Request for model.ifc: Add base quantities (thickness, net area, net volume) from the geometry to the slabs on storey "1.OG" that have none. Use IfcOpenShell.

First a look at what the model holds.

```python
import ifcopenshell
import ifcopenshell.util.element
import ifcopenshell.util.unit

model = ifcopenshell.open("model.ifc")
print(model.schema)
for unit_type in ("LENGTHUNIT", "AREAUNIT", "VOLUMEUNIT"):
    print(unit_type, ifcopenshell.util.unit.calculate_unit_scale(model, unit_type))
storey = next(s for s in model.by_type("IfcBuildingStorey") if s.Name == "1.OG")
slabs = [e for e in ifcopenshell.util.element.get_decomposition(storey) if e.is_a("IfcSlab")]
for e in sorted(slabs, key=lambda e: e.id()):
    print(e.id(), e.is_a(), e.Name, list(ifcopenshell.util.element.get_psets(e, qtos_only=True)), sep=" | ")
```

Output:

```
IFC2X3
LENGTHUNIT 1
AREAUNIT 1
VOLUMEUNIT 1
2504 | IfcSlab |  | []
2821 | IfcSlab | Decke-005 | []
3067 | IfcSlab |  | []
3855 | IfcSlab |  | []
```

```python
import ifcopenshell
import ifcopenshell.api.pset
import ifcopenshell.geom
import ifcopenshell.util.element
import ifcopenshell.util.shape
import ifcopenshell.util.unit

model = ifcopenshell.open("model.ifc")
unit_scale = ifcopenshell.util.unit.calculate_unit_scale(model)
area_scale = ifcopenshell.util.unit.calculate_unit_scale(model, "AREAUNIT")
volume_scale = ifcopenshell.util.unit.calculate_unit_scale(model, "VOLUMEUNIT")
settings = ifcopenshell.geom.settings()

storey = next(s for s in model.by_type("IfcBuildingStorey") if s.Name == "1.OG")
slabs = [e for e in ifcopenshell.util.element.get_decomposition(storey) if e.is_a("IfcSlab")]

for e in sorted(slabs, key=lambda e: e.id()):
    if ifcopenshell.util.element.get_psets(e, qtos_only=True, should_inherit=False):
        continue
    # Geometry comes back in metres, in the element's own axes.
    shape = ifcopenshell.geom.create_shape(settings, e)
    values = {
        "Width": ifcopenshell.util.shape.get_z(shape.geometry) / unit_scale,
        "NetArea": ifcopenshell.util.shape.get_footprint_area(shape.geometry) / area_scale,
        "NetVolume": ifcopenshell.util.shape.get_volume(shape.geometry) / volume_scale,
    }
    qto = ifcopenshell.api.pset.add_qto(model, product=e, name="BaseQuantities")
    ifcopenshell.api.pset.edit_qto(model, qto=qto, properties=values)
    print(e.id(), {k: round(v, 3) for k, v in values.items()})

model.write("model_updated.ifc")
```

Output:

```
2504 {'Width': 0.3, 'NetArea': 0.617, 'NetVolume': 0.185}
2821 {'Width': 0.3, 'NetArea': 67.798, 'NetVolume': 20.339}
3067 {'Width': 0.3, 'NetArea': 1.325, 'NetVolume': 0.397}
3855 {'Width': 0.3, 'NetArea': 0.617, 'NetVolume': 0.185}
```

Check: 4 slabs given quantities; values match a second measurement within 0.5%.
